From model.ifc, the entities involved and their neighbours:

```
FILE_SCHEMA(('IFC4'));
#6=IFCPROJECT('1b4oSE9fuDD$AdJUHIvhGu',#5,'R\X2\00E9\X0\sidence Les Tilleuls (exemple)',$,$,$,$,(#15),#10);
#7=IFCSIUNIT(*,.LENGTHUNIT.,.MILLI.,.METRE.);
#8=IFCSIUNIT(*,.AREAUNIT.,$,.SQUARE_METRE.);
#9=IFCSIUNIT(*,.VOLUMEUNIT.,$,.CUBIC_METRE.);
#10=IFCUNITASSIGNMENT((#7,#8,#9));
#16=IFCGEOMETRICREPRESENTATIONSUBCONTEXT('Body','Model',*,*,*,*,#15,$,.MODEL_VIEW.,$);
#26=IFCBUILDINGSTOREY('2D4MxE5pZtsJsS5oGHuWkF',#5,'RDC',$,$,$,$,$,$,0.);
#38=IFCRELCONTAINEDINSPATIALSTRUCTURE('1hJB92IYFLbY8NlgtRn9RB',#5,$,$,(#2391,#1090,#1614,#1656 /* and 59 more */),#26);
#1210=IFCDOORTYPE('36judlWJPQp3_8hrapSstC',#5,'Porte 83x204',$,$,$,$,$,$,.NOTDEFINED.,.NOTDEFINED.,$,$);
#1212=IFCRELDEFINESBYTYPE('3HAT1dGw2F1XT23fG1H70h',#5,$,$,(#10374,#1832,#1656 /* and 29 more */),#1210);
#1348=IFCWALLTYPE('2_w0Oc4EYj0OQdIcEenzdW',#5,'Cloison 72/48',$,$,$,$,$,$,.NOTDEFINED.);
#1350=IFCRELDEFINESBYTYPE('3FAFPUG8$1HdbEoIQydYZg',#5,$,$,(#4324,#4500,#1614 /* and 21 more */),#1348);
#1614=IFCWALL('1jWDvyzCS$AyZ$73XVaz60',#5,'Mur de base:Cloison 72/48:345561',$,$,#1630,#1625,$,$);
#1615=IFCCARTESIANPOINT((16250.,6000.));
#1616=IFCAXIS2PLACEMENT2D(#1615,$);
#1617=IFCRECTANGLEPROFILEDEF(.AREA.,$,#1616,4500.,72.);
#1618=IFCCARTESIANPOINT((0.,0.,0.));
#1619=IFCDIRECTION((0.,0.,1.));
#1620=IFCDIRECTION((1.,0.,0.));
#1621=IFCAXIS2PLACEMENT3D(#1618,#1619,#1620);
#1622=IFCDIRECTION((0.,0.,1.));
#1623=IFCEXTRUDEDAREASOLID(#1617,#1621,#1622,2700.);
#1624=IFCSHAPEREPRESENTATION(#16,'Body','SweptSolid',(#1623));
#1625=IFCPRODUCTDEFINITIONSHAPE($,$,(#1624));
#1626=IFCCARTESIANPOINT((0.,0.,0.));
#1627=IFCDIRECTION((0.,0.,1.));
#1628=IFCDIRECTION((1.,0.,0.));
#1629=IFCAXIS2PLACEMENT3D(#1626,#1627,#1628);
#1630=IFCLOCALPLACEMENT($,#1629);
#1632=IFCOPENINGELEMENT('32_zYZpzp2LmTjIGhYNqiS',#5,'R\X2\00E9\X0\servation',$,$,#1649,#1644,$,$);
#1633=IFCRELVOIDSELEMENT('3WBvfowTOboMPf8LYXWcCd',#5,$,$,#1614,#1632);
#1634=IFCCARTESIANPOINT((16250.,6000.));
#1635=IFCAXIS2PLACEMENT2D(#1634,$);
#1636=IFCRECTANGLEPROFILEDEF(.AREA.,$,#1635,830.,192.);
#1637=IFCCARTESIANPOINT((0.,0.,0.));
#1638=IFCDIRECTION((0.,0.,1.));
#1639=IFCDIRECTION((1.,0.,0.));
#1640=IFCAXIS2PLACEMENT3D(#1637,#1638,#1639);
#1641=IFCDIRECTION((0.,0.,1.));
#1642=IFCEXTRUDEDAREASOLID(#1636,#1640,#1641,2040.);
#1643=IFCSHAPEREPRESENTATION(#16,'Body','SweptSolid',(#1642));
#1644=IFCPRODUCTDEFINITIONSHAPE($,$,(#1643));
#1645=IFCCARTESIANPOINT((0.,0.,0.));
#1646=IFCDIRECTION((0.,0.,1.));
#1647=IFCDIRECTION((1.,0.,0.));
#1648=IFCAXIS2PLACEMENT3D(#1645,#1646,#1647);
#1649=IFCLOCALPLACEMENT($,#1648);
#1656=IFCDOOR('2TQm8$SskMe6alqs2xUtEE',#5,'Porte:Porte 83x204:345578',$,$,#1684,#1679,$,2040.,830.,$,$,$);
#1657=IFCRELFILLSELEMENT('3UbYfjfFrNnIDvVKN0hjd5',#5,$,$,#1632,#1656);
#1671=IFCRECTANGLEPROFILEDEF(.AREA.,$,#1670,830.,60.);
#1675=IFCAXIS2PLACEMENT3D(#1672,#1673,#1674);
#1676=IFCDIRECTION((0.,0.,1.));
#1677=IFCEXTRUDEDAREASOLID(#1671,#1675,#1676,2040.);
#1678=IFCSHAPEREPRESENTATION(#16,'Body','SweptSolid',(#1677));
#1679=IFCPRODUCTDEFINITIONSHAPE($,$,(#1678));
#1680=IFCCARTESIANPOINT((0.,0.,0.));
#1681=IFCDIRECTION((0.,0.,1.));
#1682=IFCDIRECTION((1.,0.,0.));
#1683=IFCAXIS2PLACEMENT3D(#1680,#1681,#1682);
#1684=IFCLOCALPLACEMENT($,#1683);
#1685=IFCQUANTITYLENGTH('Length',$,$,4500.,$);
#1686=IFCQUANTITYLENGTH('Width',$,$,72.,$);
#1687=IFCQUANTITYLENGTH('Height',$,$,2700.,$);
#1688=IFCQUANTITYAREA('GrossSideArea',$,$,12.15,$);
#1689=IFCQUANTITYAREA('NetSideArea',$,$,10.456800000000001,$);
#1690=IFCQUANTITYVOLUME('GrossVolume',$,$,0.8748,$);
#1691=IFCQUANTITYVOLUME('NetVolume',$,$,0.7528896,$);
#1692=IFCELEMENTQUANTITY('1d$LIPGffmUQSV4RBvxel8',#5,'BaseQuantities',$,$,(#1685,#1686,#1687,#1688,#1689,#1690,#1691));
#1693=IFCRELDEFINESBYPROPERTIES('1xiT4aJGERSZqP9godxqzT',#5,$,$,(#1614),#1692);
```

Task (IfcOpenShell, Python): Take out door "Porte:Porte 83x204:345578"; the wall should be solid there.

```python
import ifcopenshell
import ifcopenshell.api.feature
import ifcopenshell.api.pset
import ifcopenshell.api.root
import ifcopenshell.geom
import ifcopenshell.util.element
import ifcopenshell.util.shape
import ifcopenshell.util.unit

model = ifcopenshell.open("model.ifc")
area_scale = ifcopenshell.util.unit.calculate_unit_scale(model, "AREAUNIT")
volume_scale = ifcopenshell.util.unit.calculate_unit_scale(model, "VOLUMEUNIT")
settings = ifcopenshell.geom.settings()


def volume(element):
    """Net volume in cubic metres, openings subtracted."""
    shape = ifcopenshell.geom.create_shape(settings, element)
    return ifcopenshell.util.shape.get_volume(shape.geometry)


door = model.by_guid("2TQm8$SskMe6alqs2xUtEE")
opening = door.FillsVoids[0].RelatingOpeningElement
wall = opening.VoidsElements[0].RelatingBuildingElement
before = volume(wall)

ifcopenshell.api.root.remove_product(model, product=door)
ifcopenshell.api.feature.remove_feature(model, feature=opening)

after = volume(wall)
thickness = 0.072  # wall thickness in metres

# Update the wall's stored quantities.
qto = model.by_id(ifcopenshell.util.element.get_pset(wall, "BaseQuantities", should_inherit=False)["id"])
ifcopenshell.api.pset.edit_qto(model, qto=qto, properties={
    "NetSideArea": after / thickness / area_scale,
    "NetVolume": after / volume_scale,
})

print(f"wall volume {before:.3f} -> {after:.3f} m3")

model.write("model-out.ifc")
```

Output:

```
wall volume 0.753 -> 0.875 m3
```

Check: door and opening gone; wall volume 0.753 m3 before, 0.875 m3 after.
